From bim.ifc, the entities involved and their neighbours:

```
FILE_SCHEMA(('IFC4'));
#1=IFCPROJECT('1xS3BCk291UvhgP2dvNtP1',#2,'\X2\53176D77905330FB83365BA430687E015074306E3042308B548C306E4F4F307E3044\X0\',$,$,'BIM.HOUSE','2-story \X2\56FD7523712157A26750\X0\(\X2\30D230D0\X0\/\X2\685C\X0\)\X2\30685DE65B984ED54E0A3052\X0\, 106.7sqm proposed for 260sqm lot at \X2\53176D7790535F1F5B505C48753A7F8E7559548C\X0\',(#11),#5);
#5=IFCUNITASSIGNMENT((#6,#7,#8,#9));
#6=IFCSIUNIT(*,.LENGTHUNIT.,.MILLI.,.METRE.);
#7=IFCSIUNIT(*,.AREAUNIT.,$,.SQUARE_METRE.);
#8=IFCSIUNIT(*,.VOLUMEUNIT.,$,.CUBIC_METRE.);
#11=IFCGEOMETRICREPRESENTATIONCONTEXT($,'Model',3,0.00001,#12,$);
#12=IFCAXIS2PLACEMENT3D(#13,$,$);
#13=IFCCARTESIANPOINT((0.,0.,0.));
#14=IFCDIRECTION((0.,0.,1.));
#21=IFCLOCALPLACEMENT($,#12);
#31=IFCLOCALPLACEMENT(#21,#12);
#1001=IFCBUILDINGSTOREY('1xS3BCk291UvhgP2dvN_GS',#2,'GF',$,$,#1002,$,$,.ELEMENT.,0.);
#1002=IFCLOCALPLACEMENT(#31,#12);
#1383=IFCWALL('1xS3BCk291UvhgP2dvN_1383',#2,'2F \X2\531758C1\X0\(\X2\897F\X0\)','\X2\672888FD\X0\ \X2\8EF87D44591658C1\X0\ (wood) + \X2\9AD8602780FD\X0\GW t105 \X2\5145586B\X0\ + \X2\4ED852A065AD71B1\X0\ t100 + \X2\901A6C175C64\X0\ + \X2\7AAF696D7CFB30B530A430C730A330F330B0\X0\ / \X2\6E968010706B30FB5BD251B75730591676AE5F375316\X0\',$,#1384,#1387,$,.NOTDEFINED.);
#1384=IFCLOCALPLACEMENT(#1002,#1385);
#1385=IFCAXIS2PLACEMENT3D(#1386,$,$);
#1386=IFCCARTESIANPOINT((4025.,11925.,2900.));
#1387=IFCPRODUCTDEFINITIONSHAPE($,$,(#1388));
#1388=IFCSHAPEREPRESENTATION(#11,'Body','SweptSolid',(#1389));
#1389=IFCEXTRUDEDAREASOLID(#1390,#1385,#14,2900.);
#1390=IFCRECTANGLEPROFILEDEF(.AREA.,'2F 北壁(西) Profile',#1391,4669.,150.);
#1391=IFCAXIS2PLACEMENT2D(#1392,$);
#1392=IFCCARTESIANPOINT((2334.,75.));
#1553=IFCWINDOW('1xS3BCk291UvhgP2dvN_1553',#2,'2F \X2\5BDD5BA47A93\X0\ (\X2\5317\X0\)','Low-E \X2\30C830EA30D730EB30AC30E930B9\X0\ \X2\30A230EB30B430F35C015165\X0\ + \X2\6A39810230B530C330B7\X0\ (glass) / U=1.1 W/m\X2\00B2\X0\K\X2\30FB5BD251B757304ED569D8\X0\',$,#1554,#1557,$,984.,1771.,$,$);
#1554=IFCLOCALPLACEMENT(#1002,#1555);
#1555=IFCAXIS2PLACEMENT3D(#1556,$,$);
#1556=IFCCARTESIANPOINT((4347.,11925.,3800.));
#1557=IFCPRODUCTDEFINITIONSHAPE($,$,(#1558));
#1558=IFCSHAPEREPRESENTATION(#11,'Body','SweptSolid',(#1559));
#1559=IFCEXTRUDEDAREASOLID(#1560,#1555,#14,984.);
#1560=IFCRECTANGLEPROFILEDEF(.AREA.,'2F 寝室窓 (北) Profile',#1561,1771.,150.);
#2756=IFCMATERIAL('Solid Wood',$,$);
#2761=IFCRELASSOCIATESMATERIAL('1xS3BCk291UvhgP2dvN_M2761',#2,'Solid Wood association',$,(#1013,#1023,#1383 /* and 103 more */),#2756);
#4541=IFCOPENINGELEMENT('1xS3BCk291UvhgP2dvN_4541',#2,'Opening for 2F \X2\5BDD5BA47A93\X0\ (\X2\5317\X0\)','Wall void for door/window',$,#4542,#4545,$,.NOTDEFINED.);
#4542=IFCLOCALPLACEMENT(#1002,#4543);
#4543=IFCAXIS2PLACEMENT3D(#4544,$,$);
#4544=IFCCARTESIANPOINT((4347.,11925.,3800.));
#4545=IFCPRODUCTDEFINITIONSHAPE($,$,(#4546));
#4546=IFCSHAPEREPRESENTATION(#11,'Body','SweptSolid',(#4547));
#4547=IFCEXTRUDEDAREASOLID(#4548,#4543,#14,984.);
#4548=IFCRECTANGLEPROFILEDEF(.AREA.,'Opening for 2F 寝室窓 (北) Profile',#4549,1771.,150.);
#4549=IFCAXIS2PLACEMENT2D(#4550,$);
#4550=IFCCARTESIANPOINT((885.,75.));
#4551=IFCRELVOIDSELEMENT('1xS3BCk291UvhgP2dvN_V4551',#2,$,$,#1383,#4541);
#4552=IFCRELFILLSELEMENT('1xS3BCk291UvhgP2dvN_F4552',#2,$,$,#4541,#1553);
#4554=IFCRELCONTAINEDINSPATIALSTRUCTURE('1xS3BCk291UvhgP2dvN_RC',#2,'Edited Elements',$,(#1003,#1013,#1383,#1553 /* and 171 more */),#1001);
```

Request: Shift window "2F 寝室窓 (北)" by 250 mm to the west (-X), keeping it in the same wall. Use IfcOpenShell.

```python
import ifcopenshell
import ifcopenshell.api.geometry
import ifcopenshell.util.placement

model = ifcopenshell.open("bim.ifc")

window = model.by_guid("1xS3BCk291UvhgP2dvN_1553")
opening = window.FillsVoids[0].RelatingOpeningElement
wall = opening.VoidsElements[0].RelatingBuildingElement

wall_matrix = ifcopenshell.util.placement.get_local_placement(wall.ObjectPlacement)
shift = wall_matrix[:3, 0] * -250.0
before = ifcopenshell.util.placement.get_local_placement(window.ObjectPlacement)[:3, 3].copy()

# The window is not placed relative to its opening, so move both.
for product in (opening, window):
    matrix = ifcopenshell.util.placement.get_local_placement(product.ObjectPlacement)
    matrix[:3, 3] += shift
    ifcopenshell.api.geometry.edit_object_placement(model, product=product, matrix=matrix, is_si=False)

after = ifcopenshell.util.placement.get_local_placement(window.ObjectPlacement)[:3, 3]
print("window moved by", (after - before).round(3) + 0.0)

model.write("bim_rev.ifc")
```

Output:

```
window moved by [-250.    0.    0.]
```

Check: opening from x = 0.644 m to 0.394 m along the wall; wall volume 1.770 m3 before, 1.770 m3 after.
